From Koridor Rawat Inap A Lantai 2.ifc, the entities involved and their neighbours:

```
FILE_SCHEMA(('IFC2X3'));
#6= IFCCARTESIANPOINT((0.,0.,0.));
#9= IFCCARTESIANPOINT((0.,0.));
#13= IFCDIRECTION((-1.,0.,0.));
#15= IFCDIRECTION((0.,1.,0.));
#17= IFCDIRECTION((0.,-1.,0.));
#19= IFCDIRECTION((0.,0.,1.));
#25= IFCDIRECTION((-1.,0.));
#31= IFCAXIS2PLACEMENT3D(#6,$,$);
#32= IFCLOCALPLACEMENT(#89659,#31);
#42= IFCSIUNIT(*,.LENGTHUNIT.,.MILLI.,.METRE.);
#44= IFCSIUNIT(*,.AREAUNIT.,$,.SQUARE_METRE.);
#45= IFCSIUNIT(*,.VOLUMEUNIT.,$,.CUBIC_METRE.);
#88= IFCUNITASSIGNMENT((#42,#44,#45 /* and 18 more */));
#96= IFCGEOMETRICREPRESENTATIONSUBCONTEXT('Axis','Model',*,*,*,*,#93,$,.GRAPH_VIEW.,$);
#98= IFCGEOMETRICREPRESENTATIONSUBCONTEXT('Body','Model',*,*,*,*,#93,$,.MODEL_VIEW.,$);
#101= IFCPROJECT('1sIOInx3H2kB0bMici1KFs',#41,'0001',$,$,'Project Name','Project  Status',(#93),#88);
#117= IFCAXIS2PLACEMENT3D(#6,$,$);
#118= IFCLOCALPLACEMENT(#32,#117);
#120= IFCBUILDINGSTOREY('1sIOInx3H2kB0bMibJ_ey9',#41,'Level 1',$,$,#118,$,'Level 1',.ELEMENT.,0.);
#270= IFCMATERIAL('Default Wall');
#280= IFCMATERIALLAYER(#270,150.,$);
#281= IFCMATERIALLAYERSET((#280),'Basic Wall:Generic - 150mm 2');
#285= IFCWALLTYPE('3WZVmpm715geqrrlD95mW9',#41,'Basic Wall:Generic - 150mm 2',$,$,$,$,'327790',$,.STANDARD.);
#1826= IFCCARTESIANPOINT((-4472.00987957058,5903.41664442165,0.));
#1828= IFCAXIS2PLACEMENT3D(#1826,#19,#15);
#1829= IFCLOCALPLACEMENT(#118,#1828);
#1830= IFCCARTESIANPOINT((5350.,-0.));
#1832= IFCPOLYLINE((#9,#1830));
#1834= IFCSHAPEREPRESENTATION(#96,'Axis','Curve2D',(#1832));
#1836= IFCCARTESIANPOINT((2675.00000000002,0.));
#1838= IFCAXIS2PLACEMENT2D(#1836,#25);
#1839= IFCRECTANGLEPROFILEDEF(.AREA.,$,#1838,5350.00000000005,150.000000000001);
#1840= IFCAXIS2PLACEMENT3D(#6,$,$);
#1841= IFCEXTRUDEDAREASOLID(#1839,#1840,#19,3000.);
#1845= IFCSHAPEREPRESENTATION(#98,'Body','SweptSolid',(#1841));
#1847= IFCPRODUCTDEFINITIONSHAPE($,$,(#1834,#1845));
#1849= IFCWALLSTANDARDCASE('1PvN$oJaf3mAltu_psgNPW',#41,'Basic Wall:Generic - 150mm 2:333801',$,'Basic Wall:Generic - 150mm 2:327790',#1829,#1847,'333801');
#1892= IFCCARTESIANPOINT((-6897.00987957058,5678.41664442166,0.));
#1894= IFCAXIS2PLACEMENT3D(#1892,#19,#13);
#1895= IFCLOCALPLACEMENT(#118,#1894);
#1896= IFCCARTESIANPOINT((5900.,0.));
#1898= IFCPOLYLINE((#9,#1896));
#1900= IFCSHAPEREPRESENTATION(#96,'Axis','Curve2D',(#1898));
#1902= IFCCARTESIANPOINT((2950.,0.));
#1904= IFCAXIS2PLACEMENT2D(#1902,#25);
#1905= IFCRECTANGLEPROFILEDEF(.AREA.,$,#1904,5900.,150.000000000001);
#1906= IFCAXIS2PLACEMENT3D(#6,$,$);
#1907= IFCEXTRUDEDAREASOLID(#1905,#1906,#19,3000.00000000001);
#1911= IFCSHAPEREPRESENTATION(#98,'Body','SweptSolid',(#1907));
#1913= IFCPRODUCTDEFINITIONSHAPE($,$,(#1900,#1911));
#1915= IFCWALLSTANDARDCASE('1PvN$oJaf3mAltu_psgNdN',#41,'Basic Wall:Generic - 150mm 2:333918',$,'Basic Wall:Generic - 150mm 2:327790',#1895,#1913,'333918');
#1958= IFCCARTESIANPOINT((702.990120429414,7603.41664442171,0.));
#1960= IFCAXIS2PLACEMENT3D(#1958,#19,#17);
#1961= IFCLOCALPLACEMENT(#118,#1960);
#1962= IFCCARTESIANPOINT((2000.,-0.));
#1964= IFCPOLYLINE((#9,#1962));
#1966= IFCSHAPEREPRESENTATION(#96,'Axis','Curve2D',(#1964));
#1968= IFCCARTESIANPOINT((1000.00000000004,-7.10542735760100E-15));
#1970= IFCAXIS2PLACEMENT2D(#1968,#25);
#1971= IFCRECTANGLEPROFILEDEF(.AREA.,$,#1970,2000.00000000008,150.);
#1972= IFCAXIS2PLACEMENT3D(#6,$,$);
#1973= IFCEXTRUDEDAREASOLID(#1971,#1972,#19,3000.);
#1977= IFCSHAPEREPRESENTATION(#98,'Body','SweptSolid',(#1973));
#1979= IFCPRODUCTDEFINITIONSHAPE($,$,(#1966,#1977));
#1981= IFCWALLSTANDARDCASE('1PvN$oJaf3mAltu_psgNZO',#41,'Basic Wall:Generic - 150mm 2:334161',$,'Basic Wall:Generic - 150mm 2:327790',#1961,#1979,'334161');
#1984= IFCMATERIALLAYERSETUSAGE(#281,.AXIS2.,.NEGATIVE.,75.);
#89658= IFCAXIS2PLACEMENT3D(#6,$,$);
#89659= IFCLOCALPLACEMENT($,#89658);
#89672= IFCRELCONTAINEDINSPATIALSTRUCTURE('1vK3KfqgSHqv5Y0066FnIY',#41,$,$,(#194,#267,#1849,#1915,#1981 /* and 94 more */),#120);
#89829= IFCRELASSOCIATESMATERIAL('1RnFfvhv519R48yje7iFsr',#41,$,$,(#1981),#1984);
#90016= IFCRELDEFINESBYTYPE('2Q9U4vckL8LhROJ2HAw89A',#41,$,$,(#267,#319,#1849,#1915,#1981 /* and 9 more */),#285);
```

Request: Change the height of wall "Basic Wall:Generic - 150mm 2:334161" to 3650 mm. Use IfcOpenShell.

```python
import ifcopenshell
import ifcopenshell.geom
import ifcopenshell.util.representation
import ifcopenshell.util.shape
import ifcopenshell.util.unit

model = ifcopenshell.open("Koridor Rawat Inap A Lantai 2.ifc")
unit_scale = ifcopenshell.util.unit.calculate_unit_scale(model)
settings = ifcopenshell.geom.settings()


def volume(element):
    """Net volume in cubic metres, openings subtracted."""
    shape = ifcopenshell.geom.create_shape(settings, element)
    return ifcopenshell.util.shape.get_volume(shape.geometry)


wall = model.by_id(1981)
before = volume(wall)

body = ifcopenshell.util.representation.get_representation(wall, "Model", "Body")
solid = body.Items[0]
old_height = solid.Depth
solid.Depth = 3.65 / unit_scale
after = volume(wall)

print(f"height {old_height:g} -> {solid.Depth:g}, volume {before:.3f} -> {after:.3f} m3")

model.write("Koridor Rawat Inap A Lantai 2_updated.ifc")
```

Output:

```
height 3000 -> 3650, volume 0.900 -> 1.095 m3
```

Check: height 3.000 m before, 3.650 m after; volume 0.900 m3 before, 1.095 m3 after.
